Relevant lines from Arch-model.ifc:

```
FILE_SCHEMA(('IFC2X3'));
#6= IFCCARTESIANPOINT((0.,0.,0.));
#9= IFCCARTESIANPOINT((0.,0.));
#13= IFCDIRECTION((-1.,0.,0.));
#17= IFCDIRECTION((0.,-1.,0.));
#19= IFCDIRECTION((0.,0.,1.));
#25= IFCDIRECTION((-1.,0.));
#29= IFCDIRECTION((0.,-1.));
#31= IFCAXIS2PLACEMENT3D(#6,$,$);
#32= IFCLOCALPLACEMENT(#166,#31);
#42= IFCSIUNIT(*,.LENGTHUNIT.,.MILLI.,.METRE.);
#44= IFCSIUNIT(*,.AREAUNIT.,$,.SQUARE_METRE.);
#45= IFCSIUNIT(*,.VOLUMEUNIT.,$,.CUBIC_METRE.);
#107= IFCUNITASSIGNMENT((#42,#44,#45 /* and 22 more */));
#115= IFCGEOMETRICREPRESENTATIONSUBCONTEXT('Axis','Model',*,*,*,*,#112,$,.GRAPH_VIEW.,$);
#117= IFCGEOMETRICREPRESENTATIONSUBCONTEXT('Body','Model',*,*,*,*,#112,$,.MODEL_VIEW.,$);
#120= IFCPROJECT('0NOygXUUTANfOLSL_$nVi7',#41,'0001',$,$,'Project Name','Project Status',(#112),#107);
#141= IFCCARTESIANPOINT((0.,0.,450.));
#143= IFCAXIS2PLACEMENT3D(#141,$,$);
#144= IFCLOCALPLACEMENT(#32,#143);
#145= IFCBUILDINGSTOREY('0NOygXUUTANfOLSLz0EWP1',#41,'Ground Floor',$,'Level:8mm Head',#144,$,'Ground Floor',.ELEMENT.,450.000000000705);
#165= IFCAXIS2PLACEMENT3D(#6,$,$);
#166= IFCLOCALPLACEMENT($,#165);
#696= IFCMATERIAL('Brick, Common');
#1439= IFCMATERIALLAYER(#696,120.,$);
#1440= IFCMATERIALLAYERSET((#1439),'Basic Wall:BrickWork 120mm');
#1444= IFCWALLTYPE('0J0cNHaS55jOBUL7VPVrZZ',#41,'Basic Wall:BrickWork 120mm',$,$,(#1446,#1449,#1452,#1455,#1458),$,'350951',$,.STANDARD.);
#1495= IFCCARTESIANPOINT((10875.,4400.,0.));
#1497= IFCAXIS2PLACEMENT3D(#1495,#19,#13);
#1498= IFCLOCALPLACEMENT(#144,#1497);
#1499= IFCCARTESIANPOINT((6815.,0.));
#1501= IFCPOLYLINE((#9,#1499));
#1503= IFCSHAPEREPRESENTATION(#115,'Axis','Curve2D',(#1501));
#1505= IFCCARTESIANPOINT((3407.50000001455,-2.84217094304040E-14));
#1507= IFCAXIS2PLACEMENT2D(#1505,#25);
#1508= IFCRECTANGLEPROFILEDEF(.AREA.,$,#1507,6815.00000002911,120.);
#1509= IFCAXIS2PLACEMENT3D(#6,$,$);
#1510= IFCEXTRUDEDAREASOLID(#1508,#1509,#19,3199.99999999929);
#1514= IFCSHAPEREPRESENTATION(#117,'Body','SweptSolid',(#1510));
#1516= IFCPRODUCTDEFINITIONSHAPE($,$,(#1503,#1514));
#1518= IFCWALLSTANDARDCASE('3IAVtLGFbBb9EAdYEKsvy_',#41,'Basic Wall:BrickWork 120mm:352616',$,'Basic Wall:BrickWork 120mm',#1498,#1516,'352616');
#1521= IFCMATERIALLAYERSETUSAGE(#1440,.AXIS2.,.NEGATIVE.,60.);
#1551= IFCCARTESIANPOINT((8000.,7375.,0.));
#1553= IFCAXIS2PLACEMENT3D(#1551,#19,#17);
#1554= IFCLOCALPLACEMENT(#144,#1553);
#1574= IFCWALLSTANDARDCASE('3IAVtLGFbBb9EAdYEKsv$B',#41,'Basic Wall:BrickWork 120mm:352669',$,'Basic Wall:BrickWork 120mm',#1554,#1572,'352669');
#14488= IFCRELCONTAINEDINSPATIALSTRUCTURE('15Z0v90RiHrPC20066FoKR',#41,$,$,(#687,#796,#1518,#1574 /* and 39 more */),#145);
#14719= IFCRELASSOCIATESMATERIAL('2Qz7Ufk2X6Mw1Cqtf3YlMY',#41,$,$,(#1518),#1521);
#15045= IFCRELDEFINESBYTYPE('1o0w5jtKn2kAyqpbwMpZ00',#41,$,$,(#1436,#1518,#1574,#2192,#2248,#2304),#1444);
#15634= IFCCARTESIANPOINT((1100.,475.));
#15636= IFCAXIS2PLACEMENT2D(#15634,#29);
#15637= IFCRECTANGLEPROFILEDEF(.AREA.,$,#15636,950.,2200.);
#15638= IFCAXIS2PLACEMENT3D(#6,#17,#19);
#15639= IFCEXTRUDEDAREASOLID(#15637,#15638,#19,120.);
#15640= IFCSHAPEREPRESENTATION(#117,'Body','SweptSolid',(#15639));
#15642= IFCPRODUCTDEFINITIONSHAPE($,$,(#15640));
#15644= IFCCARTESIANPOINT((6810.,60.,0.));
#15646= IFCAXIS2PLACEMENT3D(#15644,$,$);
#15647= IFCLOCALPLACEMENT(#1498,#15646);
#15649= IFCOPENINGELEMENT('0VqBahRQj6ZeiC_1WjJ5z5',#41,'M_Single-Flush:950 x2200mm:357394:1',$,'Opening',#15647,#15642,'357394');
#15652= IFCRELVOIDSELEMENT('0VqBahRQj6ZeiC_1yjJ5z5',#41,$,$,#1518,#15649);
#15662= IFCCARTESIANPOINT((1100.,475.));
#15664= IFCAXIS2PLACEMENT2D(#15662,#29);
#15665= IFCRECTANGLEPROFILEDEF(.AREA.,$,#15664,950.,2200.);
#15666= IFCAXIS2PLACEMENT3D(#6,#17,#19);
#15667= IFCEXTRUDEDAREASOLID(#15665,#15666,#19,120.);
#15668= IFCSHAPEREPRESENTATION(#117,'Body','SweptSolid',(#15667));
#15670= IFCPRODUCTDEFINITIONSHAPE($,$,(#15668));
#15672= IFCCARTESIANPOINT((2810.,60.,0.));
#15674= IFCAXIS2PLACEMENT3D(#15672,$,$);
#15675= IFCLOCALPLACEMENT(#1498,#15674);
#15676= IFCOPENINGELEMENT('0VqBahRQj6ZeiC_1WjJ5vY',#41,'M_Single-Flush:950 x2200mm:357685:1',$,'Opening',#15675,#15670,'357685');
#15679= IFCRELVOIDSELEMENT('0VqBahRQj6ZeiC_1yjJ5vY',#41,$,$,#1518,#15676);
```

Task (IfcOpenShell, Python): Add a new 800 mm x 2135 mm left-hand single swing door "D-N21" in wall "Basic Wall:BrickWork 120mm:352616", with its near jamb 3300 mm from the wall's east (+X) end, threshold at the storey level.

```python
import numpy as np
import ifcopenshell
import ifcopenshell.api.feature
import ifcopenshell.api.geometry
import ifcopenshell.api.root
import ifcopenshell.api.spatial
import ifcopenshell.api.type
import ifcopenshell.geom
import ifcopenshell.util.element
import ifcopenshell.util.placement
import ifcopenshell.util.representation
import ifcopenshell.util.shape
import ifcopenshell.util.unit

model = ifcopenshell.open("Arch-model.ifc")
unit_scale = ifcopenshell.util.unit.calculate_unit_scale(model)
settings = ifcopenshell.geom.settings()


def volume(element):
    """Net volume in cubic metres, openings subtracted."""
    shape = ifcopenshell.geom.create_shape(settings, element)
    return ifcopenshell.util.shape.get_volume(shape.geometry)


wall = model.by_guid("3IAVtLGFbBb9EAdYEKsvy_")
storey = ifcopenshell.util.element.get_container(wall, ifc_class="IfcBuildingStorey")
context = ifcopenshell.util.representation.get_context(model, "Model", "Body", "MODEL_VIEW")
before = volume(wall)

width, height, from_end, sill = 0.8, 2.135, 3.3, 0.0  # metres

# The wall runs along its own X axis, and the end named is its -X end.
wall_shape = ifcopenshell.geom.create_shape(settings, wall)
x, y, z = ifcopenshell.util.shape.get_vertices(wall_shape.geometry).T
start = x.min() + from_end
face, thickness = float(y.min()), float(y.max() - y.min())
wall_matrix = ifcopenshell.util.placement.get_local_placement(wall.ObjectPlacement)
level = ifcopenshell.util.placement.get_local_placement(storey.ObjectPlacement)[2, 3]


def in_wall(x, y):
    """Placement at x, y metres in the wall's axes, at sill height."""
    matrix = wall_matrix.copy()
    matrix[:, 3] = wall_matrix @ np.array([x / unit_scale, y / unit_scale, 0.0, 1.0])
    matrix[2, 3] = level + sill / unit_scale
    return matrix


# Opening: a box that overshoots both wall faces by 50 mm.
opening = ifcopenshell.api.root.create_entity(model, ifc_class="IfcOpeningElement")
box = ifcopenshell.api.geometry.add_wall_representation(
    model, context=context, length=width, height=height, thickness=thickness + 0.1
)
ifcopenshell.api.geometry.assign_representation(model, product=opening, representation=box)
ifcopenshell.api.geometry.edit_object_placement(model, product=opening, matrix=in_wall(start, face - 0.05), is_si=False)
ifcopenshell.api.feature.add_feature(model, feature=opening, element=wall)

door = ifcopenshell.api.root.create_entity(model, ifc_class="IfcDoor", name="D-N21")
door.OverallWidth, door.OverallHeight = width / unit_scale, height / unit_scale
body = ifcopenshell.api.geometry.add_door_representation(
    model,
    context=context,
    overall_width=door.OverallWidth,
    overall_height=door.OverallHeight,
    operation_type="SINGLE_SWING_LEFT",
    lining_properties={"LiningDepth": thickness / unit_scale, "ThresholdDepth": thickness / unit_scale},
)
ifcopenshell.api.geometry.assign_representation(model, product=door, representation=body)
ifcopenshell.api.spatial.assign_container(model, products=[door], relating_structure=storey)
fills = ifcopenshell.api.feature.add_filling(model, opening=opening, element=door)
fills.OwnerHistory = door.OwnerHistory  # required in IFC2X3

# IFC2X3 keeps the operation on the door style.
style = ifcopenshell.api.root.create_entity(model, ifc_class="IfcDoorStyle", name="D-N21")
style.OperationType, style.ConstructionType = "SINGLE_SWING_LEFT", "NOTDEFINED"
style.ParameterTakesPrecedence = style.Sizeable = False
ifcopenshell.api.type.assign_type(model, related_objects=[door], relating_type=style)

# The lining spans the wall, so the door starts at the wall face.
ifcopenshell.api.geometry.edit_object_placement(model, product=door, matrix=in_wall(start, face), is_si=False)

after = volume(wall)

print(f"wall volume {before:.3f} -> {after:.3f} m3")

model.write("Arch-model_v2.ifc")
```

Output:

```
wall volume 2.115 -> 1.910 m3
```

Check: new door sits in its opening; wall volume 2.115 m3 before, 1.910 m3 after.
